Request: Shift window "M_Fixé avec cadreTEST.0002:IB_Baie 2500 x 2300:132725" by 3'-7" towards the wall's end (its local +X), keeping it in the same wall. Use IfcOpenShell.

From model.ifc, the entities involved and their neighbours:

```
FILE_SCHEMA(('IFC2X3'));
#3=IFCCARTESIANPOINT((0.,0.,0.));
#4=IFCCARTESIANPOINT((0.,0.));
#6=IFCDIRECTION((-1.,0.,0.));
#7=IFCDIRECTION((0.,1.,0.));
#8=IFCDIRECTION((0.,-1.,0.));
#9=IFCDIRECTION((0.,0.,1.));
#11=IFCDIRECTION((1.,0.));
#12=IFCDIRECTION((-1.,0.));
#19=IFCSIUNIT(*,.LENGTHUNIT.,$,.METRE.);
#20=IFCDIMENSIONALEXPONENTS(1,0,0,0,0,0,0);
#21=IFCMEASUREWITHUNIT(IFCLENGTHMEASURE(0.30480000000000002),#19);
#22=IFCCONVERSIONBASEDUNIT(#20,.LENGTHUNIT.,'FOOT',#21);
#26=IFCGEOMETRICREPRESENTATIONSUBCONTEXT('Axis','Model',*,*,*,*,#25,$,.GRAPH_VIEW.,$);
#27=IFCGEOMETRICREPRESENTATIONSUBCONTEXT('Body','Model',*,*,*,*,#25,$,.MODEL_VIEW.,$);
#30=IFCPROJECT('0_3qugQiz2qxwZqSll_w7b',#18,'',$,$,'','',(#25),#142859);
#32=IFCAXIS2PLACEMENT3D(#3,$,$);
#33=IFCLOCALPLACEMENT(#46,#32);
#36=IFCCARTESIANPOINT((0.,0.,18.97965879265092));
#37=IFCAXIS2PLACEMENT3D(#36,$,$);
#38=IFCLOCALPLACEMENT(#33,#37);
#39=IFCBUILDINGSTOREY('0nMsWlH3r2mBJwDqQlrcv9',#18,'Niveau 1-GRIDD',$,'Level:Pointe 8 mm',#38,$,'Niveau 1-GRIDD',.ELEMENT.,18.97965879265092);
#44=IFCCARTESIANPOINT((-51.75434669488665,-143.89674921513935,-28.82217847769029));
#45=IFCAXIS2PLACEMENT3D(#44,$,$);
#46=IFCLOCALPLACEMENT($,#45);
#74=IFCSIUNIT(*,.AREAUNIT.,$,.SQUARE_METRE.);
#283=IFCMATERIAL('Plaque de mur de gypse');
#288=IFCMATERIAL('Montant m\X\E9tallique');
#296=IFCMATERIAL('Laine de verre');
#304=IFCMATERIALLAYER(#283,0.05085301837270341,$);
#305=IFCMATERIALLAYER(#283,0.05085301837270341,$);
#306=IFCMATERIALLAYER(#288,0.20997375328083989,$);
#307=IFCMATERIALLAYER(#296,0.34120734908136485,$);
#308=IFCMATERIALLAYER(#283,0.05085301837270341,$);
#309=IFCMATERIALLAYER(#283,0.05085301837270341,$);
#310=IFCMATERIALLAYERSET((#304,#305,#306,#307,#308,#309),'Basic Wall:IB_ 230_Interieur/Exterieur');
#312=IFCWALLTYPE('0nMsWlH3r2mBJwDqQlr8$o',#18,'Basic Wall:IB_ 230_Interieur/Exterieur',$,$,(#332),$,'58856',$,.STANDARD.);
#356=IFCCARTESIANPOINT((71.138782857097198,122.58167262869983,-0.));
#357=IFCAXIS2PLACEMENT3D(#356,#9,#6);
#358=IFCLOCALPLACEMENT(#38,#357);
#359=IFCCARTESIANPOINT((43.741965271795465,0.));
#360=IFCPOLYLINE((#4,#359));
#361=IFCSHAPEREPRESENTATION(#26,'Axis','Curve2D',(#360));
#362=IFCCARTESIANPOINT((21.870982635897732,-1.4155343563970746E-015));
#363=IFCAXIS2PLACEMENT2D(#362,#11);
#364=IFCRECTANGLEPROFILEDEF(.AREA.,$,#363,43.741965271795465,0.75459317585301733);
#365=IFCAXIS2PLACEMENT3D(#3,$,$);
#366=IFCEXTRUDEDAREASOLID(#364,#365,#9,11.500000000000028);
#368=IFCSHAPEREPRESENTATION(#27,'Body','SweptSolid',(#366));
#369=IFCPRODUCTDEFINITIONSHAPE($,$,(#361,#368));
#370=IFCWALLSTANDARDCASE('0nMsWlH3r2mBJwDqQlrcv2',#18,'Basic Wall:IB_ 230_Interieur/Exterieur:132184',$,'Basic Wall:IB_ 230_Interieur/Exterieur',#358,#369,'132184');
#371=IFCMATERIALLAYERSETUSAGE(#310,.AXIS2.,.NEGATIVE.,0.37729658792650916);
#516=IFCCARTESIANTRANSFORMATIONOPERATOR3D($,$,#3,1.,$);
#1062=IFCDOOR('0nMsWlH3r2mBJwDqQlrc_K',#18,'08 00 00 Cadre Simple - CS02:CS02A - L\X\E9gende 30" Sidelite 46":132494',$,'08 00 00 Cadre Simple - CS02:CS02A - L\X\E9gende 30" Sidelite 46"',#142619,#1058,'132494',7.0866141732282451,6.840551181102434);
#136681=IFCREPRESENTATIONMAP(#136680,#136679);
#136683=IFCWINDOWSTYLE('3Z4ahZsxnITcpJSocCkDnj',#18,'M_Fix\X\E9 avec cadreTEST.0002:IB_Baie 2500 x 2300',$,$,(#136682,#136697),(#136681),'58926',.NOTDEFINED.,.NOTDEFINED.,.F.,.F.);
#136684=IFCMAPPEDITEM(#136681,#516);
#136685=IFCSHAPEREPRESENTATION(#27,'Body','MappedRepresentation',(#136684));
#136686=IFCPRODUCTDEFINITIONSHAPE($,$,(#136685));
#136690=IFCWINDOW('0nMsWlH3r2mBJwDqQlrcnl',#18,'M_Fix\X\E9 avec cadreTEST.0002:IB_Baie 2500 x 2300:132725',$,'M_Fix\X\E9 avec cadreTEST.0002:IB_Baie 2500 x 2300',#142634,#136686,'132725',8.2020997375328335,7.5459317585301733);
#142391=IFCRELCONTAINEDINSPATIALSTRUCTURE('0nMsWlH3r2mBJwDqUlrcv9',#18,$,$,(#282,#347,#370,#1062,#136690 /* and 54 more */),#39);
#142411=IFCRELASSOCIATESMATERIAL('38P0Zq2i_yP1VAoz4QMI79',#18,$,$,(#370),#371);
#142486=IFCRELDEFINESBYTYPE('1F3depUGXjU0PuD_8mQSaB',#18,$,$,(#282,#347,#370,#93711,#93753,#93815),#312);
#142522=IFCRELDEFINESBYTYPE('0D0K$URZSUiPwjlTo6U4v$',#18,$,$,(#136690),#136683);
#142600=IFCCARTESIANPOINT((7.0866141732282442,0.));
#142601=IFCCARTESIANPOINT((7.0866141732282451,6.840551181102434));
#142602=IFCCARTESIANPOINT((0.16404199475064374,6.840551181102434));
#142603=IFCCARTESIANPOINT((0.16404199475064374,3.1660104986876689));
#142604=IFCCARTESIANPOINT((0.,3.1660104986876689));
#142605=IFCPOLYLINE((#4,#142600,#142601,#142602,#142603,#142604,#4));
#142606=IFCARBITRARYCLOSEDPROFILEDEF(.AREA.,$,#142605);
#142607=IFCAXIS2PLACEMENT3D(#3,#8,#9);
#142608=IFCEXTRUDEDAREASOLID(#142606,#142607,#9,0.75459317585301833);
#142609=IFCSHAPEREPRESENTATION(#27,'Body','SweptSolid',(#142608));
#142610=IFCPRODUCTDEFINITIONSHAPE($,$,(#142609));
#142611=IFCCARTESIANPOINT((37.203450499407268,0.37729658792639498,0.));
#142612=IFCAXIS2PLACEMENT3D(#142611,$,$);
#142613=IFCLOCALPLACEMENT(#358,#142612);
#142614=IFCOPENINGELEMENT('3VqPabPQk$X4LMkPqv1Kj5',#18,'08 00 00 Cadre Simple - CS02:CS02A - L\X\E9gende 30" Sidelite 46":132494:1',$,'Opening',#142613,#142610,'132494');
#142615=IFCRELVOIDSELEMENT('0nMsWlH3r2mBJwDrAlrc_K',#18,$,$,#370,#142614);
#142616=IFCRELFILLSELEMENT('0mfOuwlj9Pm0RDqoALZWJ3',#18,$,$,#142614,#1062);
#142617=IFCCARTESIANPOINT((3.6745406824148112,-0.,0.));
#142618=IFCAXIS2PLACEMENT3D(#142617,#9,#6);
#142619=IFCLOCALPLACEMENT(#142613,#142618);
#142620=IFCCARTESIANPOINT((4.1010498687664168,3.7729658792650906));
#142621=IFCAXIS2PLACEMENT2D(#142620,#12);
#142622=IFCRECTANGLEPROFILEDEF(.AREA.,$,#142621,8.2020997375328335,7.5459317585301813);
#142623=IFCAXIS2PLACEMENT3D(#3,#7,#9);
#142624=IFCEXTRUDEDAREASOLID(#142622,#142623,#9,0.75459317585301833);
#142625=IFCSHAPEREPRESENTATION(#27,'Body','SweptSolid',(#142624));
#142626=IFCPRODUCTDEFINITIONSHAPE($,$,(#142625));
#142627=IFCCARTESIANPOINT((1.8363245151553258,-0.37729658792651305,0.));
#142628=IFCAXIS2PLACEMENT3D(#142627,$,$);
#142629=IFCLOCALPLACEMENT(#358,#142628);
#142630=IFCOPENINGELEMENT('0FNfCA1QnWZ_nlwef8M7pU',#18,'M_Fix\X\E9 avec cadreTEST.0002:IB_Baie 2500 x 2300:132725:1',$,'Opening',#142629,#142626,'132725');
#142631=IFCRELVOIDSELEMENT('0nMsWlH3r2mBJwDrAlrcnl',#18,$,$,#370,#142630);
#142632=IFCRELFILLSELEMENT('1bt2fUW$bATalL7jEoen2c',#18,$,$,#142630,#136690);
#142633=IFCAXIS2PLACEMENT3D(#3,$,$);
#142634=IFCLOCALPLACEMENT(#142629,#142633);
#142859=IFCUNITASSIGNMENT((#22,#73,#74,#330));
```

```python
import ifcopenshell
import ifcopenshell.api.geometry
import ifcopenshell.util.placement
import ifcopenshell.util.unit

model = ifcopenshell.open("model.ifc")
unit_scale = ifcopenshell.util.unit.calculate_unit_scale(model)

window = model.by_id(136690)
opening = window.FillsVoids[0].RelatingOpeningElement
wall = opening.VoidsElements[0].RelatingBuildingElement

wall_matrix = ifcopenshell.util.placement.get_local_placement(wall.ObjectPlacement)
shift = wall_matrix[:3, 0] * 43 * 0.0254 / unit_scale
before = ifcopenshell.util.placement.get_local_placement(window.ObjectPlacement)[:3, 3].copy()

# The window is placed relative to its opening, so it follows when the opening moves.
matrix = ifcopenshell.util.placement.get_local_placement(opening.ObjectPlacement)
matrix[:3, 3] += shift
ifcopenshell.api.geometry.edit_object_placement(
    model, product=opening, matrix=matrix, is_si=False, should_transform_children=True
)

after = ifcopenshell.util.placement.get_local_placement(window.ObjectPlacement)[:3, 3]
print("window moved by", (after - before).round(3) + 0.0)

model.write("model_rev.ifc")
```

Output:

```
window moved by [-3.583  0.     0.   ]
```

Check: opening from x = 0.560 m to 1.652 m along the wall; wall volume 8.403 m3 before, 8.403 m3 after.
